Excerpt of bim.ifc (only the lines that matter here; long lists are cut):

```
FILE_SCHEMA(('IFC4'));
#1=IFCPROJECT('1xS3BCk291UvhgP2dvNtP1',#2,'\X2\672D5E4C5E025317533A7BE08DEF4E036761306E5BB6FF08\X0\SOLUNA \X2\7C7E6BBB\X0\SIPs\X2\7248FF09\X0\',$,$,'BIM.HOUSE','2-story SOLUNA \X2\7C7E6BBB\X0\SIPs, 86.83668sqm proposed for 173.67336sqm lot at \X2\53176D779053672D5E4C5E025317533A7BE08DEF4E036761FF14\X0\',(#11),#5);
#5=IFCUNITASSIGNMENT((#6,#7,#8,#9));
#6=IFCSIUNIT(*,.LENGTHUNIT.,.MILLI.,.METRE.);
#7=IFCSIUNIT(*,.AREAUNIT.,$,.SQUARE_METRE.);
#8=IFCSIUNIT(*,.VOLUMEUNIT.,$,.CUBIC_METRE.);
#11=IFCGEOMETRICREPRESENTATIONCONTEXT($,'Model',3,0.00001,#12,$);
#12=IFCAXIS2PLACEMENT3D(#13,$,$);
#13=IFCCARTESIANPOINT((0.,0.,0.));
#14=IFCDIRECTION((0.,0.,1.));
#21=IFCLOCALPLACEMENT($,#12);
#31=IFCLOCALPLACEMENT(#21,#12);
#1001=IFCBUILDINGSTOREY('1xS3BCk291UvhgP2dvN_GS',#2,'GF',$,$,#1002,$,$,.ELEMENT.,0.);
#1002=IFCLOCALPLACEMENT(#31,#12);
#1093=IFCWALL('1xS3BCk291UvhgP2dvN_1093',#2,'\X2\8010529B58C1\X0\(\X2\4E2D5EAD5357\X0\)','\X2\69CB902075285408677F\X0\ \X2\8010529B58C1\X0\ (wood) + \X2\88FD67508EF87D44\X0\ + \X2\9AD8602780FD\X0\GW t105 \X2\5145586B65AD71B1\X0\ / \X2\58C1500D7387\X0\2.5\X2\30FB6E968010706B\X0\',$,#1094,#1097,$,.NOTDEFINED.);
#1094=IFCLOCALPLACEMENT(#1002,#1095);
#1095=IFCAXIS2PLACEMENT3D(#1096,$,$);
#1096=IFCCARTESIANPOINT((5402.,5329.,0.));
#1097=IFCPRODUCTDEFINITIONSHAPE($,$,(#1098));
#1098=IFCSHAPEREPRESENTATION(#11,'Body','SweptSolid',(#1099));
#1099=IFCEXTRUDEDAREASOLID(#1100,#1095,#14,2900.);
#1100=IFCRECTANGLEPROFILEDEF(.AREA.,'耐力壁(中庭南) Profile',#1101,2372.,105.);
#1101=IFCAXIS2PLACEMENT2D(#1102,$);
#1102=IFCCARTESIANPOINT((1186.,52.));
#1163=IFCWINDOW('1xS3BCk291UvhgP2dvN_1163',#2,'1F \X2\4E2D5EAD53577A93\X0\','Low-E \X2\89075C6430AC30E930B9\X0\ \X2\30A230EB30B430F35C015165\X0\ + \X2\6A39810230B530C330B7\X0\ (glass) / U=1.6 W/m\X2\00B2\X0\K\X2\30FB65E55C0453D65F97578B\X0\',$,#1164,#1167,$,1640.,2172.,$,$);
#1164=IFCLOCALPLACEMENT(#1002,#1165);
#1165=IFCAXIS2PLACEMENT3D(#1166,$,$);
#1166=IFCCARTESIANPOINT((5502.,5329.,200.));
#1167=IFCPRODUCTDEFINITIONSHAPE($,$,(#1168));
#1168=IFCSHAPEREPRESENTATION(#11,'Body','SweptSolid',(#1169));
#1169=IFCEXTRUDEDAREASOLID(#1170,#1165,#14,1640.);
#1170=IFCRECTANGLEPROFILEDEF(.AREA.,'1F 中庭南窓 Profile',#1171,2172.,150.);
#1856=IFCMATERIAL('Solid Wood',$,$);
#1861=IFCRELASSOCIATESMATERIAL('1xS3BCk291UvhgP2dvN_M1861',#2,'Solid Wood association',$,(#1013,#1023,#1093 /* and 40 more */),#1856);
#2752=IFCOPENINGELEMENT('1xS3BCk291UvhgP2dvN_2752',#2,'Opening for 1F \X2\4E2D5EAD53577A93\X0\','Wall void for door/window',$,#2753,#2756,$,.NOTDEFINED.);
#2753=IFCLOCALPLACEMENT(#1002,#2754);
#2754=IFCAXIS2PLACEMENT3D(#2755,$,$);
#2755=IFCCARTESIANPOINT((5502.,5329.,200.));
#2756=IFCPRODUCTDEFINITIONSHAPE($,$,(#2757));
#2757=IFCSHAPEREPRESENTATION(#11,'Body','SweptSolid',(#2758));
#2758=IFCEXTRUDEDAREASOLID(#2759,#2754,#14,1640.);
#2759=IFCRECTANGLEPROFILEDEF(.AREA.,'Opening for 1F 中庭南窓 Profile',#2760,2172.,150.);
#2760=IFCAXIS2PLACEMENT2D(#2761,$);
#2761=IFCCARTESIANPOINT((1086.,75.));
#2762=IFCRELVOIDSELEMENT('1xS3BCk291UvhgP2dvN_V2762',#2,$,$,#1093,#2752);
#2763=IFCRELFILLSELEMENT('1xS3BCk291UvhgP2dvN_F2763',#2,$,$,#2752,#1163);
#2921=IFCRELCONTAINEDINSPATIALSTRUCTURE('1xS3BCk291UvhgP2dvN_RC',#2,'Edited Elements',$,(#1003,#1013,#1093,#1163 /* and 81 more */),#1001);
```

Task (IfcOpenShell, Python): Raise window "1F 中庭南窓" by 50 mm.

```python
import numpy as np
import ifcopenshell
import ifcopenshell.api.geometry
import ifcopenshell.util.placement
import ifcopenshell.util.unit

model = ifcopenshell.open("bim.ifc")
unit_scale = ifcopenshell.util.unit.calculate_unit_scale(model)

window = model.by_guid("1xS3BCk291UvhgP2dvN_1163")
opening = window.FillsVoids[0].RelatingOpeningElement
dz = 0.05 / unit_scale

shift = np.array([0.0, 0.0, dz])
# The window is not placed relative to its opening, so move both.
for product in (opening, window):
    matrix = ifcopenshell.util.placement.get_local_placement(product.ObjectPlacement)
    matrix[:3, 3] += shift
    ifcopenshell.api.geometry.edit_object_placement(model, product=product, matrix=matrix, is_si=False)

print(f"moved by {dz * unit_scale:+.3f} m")

model.write("bim_updated.ifc")
```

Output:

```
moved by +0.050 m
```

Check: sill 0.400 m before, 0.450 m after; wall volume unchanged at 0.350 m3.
